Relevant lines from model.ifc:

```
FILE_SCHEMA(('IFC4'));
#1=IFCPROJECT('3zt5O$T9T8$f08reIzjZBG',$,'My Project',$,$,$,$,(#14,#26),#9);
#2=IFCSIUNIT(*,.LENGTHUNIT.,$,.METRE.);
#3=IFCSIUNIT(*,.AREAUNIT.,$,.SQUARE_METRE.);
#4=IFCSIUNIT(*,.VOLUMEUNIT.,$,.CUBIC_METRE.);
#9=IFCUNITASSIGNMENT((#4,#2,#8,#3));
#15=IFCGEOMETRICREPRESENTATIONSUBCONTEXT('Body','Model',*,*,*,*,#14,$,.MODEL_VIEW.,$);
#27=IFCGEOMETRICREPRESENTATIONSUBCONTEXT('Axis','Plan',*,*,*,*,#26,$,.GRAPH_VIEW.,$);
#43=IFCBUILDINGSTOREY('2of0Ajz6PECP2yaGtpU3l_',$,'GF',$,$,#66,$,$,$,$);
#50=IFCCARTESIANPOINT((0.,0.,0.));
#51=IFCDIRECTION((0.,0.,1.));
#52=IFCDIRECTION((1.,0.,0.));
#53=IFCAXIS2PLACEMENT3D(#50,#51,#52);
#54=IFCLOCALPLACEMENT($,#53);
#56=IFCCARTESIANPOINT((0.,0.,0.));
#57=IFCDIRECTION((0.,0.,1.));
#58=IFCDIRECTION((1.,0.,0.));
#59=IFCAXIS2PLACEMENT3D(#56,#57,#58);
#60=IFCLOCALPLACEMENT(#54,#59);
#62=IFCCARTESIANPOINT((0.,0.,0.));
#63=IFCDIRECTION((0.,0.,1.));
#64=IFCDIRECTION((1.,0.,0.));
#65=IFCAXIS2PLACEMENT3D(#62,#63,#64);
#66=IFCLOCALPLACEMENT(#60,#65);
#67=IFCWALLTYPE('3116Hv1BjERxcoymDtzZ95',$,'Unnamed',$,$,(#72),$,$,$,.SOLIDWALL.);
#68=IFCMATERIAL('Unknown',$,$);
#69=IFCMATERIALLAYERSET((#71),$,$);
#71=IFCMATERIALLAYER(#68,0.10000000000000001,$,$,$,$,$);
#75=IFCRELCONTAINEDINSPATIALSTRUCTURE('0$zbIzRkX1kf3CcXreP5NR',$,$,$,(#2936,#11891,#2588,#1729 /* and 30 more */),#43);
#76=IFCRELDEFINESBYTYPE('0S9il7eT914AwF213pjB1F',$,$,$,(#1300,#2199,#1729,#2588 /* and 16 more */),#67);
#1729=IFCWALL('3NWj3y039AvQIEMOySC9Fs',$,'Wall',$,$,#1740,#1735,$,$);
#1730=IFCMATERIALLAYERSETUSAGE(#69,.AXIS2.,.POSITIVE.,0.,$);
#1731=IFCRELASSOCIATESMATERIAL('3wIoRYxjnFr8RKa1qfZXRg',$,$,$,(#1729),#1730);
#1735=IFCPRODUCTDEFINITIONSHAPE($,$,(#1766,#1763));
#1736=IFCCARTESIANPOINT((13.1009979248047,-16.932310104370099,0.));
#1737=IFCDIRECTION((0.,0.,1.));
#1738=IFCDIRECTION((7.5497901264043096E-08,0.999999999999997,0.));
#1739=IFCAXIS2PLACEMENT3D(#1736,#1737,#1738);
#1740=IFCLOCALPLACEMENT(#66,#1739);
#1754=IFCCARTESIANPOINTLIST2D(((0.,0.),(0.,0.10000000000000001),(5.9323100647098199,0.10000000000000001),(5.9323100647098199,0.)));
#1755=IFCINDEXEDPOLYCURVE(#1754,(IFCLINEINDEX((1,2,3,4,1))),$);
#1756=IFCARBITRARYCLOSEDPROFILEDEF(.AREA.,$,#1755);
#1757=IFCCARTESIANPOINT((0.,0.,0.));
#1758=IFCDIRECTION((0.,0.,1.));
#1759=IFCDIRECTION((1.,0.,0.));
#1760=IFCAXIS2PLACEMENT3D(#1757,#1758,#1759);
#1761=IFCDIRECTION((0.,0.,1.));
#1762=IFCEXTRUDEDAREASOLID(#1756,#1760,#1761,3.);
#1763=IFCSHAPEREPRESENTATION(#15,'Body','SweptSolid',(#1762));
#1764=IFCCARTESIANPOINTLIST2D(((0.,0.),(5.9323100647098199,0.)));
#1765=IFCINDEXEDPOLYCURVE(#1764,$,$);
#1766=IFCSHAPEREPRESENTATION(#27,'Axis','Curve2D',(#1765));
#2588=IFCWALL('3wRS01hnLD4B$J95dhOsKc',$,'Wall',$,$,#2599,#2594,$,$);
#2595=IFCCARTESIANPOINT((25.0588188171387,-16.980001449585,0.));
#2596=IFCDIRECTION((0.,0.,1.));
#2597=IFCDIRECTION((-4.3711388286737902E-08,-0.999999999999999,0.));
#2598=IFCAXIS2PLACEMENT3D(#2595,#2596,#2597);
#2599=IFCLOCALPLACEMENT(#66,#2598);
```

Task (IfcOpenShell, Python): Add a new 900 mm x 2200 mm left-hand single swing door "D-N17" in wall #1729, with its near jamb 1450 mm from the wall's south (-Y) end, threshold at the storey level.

```python
import numpy as np
import ifcopenshell
import ifcopenshell.api.feature
import ifcopenshell.api.geometry
import ifcopenshell.api.root
import ifcopenshell.api.spatial
import ifcopenshell.geom
import ifcopenshell.util.element
import ifcopenshell.util.placement
import ifcopenshell.util.representation
import ifcopenshell.util.shape
import ifcopenshell.util.unit

model = ifcopenshell.open("model.ifc")
unit_scale = ifcopenshell.util.unit.calculate_unit_scale(model)
settings = ifcopenshell.geom.settings()


def volume(element):
    """Net volume in cubic metres, openings subtracted."""
    shape = ifcopenshell.geom.create_shape(settings, element)
    return ifcopenshell.util.shape.get_volume(shape.geometry)


wall = model.by_id(1729)
storey = ifcopenshell.util.element.get_container(wall, ifc_class="IfcBuildingStorey")
context = ifcopenshell.util.representation.get_context(model, "Model", "Body", "MODEL_VIEW")
before = volume(wall)

width, height, from_end, sill = 0.9, 2.2, 1.45, 0.0  # metres

# The wall runs along its own X axis, and the end named is its -X end.
wall_shape = ifcopenshell.geom.create_shape(settings, wall)
x, y, z = ifcopenshell.util.shape.get_vertices(wall_shape.geometry).T
start = x.min() + from_end
face, thickness = float(y.min()), float(y.max() - y.min())
wall_matrix = ifcopenshell.util.placement.get_local_placement(wall.ObjectPlacement)
level = ifcopenshell.util.placement.get_local_placement(storey.ObjectPlacement)[2, 3]


def in_wall(x, y):
    """Placement at x, y metres in the wall's axes, at sill height."""
    matrix = wall_matrix.copy()
    matrix[:, 3] = wall_matrix @ np.array([x / unit_scale, y / unit_scale, 0.0, 1.0])
    matrix[2, 3] = level + sill / unit_scale
    return matrix


# Opening: a box that overshoots both wall faces by 50 mm.
opening = ifcopenshell.api.root.create_entity(model, ifc_class="IfcOpeningElement", predefined_type="OPENING")
box = ifcopenshell.api.geometry.add_wall_representation(
    model, context=context, length=width, height=height, thickness=thickness + 0.1
)
ifcopenshell.api.geometry.assign_representation(model, product=opening, representation=box)
ifcopenshell.api.geometry.edit_object_placement(model, product=opening, matrix=in_wall(start, face - 0.05), is_si=False)
ifcopenshell.api.feature.add_feature(model, feature=opening, element=wall)

door = ifcopenshell.api.root.create_entity(model, ifc_class="IfcDoor", name="D-N17", predefined_type="DOOR")
door.OverallWidth, door.OverallHeight = width / unit_scale, height / unit_scale
door.OperationType = "SINGLE_SWING_LEFT"
body = ifcopenshell.api.geometry.add_door_representation(
    model,
    context=context,
    overall_width=door.OverallWidth,
    overall_height=door.OverallHeight,
    operation_type="SINGLE_SWING_LEFT",
    lining_properties={"LiningDepth": thickness / unit_scale, "ThresholdDepth": thickness / unit_scale},
)
ifcopenshell.api.geometry.assign_representation(model, product=door, representation=body)
ifcopenshell.api.spatial.assign_container(model, products=[door], relating_structure=storey)
ifcopenshell.api.feature.add_filling(model, opening=opening, element=door)

# The lining spans the wall, so the door starts at the wall face.
ifcopenshell.api.geometry.edit_object_placement(model, product=door, matrix=in_wall(start, face), is_si=False)

after = volume(wall)

print(f"wall volume {before:.3f} -> {after:.3f} m3")

model.write("model-out.ifc")
```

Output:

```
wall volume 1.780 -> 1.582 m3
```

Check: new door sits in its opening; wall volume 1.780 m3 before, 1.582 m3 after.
